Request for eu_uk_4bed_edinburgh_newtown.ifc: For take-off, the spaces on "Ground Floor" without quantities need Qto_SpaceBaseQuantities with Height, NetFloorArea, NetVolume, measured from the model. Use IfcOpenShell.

First a look at what the model holds.

```python
import ifcopenshell
import ifcopenshell.util.element
import ifcopenshell.util.unit

model = ifcopenshell.open("eu_uk_4bed_edinburgh_newtown.ifc")
print(model.schema)
for unit_type in ("LENGTHUNIT", "AREAUNIT", "VOLUMEUNIT"):
    print(unit_type, ifcopenshell.util.unit.calculate_unit_scale(model, unit_type))
storey = next(s for s in model.by_type("IfcBuildingStorey") if s.Name == "Ground Floor")
spaces = [e for e in ifcopenshell.util.element.get_decomposition(storey) if e.is_a("IfcSpace")]
for e in sorted(spaces, key=lambda e: e.id()):
    print(e.id(), e.is_a(), e.Name, list(ifcopenshell.util.element.get_psets(e, qtos_only=True)), sep=" | ")
```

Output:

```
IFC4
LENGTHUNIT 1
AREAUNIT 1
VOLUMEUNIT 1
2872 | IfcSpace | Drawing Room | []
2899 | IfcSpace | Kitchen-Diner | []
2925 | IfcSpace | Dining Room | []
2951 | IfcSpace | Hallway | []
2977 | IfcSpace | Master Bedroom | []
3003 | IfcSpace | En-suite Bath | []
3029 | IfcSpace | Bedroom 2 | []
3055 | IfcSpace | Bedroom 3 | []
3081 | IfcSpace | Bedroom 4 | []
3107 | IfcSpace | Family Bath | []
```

```python
import ifcopenshell
import ifcopenshell.api.pset
import ifcopenshell.geom
import ifcopenshell.util.element
import ifcopenshell.util.shape
import ifcopenshell.util.unit

model = ifcopenshell.open("eu_uk_4bed_edinburgh_newtown.ifc")
unit_scale = ifcopenshell.util.unit.calculate_unit_scale(model)
area_scale = ifcopenshell.util.unit.calculate_unit_scale(model, "AREAUNIT")
volume_scale = ifcopenshell.util.unit.calculate_unit_scale(model, "VOLUMEUNIT")
settings = ifcopenshell.geom.settings()

storey = next(s for s in model.by_type("IfcBuildingStorey") if s.Name == "Ground Floor")
spaces = [e for e in ifcopenshell.util.element.get_decomposition(storey) if e.is_a("IfcSpace")]

for e in sorted(spaces, key=lambda e: e.id()):
    if ifcopenshell.util.element.get_psets(e, qtos_only=True, should_inherit=False):
        continue
    # Geometry comes back in metres, in the element's own axes.
    shape = ifcopenshell.geom.create_shape(settings, e)
    values = {
        "Height": ifcopenshell.util.shape.get_z(shape.geometry) / unit_scale,
        "NetFloorArea": ifcopenshell.util.shape.get_footprint_area(shape.geometry) / area_scale,
        "NetVolume": ifcopenshell.util.shape.get_volume(shape.geometry) / volume_scale,
    }
    qto = ifcopenshell.api.pset.add_qto(model, product=e, name="Qto_SpaceBaseQuantities")
    ifcopenshell.api.pset.edit_qto(model, qto=qto, properties=values)
    print(e.id(), {k: round(v, 3) for k, v in values.items()})

model.write("eu_uk_4bed_edinburgh_newtown_edited.ifc")
```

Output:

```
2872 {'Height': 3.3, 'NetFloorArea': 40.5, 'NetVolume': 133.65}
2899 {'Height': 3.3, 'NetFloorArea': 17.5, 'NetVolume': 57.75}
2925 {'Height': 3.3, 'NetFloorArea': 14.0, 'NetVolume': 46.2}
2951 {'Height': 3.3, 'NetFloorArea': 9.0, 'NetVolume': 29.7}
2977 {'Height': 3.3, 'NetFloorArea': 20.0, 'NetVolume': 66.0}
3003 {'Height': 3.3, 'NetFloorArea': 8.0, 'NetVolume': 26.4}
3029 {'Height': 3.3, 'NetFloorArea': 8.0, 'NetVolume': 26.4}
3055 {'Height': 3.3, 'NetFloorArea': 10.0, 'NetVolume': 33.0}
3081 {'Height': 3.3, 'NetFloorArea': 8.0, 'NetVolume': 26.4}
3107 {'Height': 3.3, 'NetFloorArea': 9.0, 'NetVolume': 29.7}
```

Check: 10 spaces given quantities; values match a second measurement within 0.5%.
